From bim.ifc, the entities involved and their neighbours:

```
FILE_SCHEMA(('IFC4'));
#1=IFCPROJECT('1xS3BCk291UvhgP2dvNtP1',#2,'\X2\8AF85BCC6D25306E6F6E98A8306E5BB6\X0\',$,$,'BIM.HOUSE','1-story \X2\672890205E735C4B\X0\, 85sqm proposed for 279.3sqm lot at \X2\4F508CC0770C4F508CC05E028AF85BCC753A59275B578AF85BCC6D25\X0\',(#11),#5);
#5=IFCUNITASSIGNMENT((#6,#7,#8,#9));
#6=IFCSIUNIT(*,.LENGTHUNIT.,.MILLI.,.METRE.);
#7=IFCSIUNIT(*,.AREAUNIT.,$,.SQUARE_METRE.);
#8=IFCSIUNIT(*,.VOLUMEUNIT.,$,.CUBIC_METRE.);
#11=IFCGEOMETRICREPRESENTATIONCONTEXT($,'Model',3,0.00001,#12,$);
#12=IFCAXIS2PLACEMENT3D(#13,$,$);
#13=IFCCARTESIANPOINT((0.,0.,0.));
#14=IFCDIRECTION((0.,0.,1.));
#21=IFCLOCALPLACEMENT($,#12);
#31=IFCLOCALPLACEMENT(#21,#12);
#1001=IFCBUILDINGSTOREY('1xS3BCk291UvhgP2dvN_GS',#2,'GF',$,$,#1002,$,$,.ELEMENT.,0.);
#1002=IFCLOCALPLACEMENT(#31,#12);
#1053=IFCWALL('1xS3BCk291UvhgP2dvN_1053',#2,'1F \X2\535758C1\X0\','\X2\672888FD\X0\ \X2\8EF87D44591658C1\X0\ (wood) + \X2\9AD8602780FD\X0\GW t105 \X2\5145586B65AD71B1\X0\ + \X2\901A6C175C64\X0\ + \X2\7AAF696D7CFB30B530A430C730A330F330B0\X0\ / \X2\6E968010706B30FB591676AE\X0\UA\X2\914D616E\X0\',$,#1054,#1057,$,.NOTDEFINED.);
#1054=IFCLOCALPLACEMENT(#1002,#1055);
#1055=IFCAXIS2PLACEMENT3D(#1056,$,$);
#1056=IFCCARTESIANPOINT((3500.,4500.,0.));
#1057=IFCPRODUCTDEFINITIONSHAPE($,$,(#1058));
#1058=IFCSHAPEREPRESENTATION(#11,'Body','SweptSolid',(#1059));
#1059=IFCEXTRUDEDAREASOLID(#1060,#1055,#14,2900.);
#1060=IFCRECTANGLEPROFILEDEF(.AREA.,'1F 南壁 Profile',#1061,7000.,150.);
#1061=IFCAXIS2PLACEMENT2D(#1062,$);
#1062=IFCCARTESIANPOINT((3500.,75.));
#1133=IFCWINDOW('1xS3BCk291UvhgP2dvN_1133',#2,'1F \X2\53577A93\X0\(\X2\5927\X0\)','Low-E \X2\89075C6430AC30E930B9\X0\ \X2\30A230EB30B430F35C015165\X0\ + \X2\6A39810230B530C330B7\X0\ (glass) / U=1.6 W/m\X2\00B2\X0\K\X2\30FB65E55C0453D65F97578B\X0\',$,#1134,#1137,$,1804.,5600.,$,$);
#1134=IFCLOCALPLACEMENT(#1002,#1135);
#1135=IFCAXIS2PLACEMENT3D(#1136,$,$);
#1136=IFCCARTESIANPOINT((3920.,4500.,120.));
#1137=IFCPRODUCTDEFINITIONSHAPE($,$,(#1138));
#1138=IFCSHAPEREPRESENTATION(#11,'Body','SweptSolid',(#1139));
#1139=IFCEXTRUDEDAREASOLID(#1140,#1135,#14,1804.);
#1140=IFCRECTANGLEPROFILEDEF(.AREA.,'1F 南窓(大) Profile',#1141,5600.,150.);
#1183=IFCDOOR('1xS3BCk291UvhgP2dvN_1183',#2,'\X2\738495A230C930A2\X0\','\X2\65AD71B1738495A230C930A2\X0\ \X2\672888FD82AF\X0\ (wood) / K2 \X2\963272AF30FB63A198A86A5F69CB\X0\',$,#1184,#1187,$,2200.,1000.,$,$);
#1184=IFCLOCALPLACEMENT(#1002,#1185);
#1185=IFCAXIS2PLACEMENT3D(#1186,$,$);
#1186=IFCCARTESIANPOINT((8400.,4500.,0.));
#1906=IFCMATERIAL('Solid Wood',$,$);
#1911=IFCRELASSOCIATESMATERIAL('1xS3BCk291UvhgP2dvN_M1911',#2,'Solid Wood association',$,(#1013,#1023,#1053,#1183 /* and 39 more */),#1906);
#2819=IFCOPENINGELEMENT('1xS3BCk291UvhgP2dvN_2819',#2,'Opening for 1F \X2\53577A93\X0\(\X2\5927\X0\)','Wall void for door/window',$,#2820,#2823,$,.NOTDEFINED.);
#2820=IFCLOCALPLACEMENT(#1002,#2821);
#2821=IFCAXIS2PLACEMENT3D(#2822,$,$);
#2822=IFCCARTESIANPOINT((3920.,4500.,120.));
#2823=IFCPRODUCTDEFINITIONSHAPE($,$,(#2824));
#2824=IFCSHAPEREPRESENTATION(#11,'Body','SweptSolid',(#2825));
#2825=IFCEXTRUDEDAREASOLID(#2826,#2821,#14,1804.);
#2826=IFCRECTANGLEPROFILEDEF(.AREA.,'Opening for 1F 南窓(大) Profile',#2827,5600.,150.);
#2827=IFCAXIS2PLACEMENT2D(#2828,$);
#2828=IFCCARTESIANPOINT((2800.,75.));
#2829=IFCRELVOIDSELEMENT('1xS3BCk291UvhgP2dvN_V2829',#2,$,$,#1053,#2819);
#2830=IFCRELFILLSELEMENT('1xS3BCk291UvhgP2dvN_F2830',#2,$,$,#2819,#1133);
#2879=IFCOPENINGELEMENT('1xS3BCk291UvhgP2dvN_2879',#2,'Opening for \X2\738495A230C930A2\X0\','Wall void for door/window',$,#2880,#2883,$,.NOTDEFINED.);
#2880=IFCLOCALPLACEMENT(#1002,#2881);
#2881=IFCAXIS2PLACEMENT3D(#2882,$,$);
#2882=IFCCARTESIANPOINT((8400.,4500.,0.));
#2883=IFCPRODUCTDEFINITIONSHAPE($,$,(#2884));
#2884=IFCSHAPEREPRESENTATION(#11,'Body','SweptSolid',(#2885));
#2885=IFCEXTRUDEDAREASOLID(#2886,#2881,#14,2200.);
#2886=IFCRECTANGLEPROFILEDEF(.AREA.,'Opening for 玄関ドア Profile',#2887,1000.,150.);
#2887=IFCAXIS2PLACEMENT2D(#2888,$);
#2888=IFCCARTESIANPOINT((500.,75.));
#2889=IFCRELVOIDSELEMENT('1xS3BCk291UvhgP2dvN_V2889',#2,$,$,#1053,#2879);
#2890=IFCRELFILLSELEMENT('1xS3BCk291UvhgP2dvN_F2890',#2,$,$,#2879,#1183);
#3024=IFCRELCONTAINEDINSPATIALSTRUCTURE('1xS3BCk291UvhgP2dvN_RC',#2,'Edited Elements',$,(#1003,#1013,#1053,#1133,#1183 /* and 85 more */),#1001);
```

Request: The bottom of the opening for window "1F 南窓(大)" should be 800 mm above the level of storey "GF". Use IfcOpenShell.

```python
import numpy as np
import ifcopenshell
import ifcopenshell.api.geometry
import ifcopenshell.geom
import ifcopenshell.util.element
import ifcopenshell.util.placement
import ifcopenshell.util.shape
import ifcopenshell.util.unit

model = ifcopenshell.open("bim.ifc")
unit_scale = ifcopenshell.util.unit.calculate_unit_scale(model)

window = model.by_id(1133)
opening = window.FillsVoids[0].RelatingOpeningElement
storey = ifcopenshell.util.element.get_container(window, ifc_class="IfcBuildingStorey")
level = ifcopenshell.util.placement.get_local_placement(storey.ObjectPlacement)[2, 3]

# The opening's origin need not be at the sill, so measure its lowest point.
shape = ifcopenshell.geom.create_shape(ifcopenshell.geom.settings(), opening)
bottom = ifcopenshell.util.shape.get_shape_bottom_elevation(shape, shape.geometry) / unit_scale
dz = level + 0.8 / unit_scale - bottom

shift = np.array([0.0, 0.0, dz])
# The window is not placed relative to its opening, so move both.
for product in (opening, window):
    matrix = ifcopenshell.util.placement.get_local_placement(product.ObjectPlacement)
    matrix[:3, 3] += shift
    ifcopenshell.api.geometry.edit_object_placement(model, product=product, matrix=matrix, is_si=False)

print(f"moved by {dz * unit_scale:+.3f} m")

model.write("bim_updated.ifc")
```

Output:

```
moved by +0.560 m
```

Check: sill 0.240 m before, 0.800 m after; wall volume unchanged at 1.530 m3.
